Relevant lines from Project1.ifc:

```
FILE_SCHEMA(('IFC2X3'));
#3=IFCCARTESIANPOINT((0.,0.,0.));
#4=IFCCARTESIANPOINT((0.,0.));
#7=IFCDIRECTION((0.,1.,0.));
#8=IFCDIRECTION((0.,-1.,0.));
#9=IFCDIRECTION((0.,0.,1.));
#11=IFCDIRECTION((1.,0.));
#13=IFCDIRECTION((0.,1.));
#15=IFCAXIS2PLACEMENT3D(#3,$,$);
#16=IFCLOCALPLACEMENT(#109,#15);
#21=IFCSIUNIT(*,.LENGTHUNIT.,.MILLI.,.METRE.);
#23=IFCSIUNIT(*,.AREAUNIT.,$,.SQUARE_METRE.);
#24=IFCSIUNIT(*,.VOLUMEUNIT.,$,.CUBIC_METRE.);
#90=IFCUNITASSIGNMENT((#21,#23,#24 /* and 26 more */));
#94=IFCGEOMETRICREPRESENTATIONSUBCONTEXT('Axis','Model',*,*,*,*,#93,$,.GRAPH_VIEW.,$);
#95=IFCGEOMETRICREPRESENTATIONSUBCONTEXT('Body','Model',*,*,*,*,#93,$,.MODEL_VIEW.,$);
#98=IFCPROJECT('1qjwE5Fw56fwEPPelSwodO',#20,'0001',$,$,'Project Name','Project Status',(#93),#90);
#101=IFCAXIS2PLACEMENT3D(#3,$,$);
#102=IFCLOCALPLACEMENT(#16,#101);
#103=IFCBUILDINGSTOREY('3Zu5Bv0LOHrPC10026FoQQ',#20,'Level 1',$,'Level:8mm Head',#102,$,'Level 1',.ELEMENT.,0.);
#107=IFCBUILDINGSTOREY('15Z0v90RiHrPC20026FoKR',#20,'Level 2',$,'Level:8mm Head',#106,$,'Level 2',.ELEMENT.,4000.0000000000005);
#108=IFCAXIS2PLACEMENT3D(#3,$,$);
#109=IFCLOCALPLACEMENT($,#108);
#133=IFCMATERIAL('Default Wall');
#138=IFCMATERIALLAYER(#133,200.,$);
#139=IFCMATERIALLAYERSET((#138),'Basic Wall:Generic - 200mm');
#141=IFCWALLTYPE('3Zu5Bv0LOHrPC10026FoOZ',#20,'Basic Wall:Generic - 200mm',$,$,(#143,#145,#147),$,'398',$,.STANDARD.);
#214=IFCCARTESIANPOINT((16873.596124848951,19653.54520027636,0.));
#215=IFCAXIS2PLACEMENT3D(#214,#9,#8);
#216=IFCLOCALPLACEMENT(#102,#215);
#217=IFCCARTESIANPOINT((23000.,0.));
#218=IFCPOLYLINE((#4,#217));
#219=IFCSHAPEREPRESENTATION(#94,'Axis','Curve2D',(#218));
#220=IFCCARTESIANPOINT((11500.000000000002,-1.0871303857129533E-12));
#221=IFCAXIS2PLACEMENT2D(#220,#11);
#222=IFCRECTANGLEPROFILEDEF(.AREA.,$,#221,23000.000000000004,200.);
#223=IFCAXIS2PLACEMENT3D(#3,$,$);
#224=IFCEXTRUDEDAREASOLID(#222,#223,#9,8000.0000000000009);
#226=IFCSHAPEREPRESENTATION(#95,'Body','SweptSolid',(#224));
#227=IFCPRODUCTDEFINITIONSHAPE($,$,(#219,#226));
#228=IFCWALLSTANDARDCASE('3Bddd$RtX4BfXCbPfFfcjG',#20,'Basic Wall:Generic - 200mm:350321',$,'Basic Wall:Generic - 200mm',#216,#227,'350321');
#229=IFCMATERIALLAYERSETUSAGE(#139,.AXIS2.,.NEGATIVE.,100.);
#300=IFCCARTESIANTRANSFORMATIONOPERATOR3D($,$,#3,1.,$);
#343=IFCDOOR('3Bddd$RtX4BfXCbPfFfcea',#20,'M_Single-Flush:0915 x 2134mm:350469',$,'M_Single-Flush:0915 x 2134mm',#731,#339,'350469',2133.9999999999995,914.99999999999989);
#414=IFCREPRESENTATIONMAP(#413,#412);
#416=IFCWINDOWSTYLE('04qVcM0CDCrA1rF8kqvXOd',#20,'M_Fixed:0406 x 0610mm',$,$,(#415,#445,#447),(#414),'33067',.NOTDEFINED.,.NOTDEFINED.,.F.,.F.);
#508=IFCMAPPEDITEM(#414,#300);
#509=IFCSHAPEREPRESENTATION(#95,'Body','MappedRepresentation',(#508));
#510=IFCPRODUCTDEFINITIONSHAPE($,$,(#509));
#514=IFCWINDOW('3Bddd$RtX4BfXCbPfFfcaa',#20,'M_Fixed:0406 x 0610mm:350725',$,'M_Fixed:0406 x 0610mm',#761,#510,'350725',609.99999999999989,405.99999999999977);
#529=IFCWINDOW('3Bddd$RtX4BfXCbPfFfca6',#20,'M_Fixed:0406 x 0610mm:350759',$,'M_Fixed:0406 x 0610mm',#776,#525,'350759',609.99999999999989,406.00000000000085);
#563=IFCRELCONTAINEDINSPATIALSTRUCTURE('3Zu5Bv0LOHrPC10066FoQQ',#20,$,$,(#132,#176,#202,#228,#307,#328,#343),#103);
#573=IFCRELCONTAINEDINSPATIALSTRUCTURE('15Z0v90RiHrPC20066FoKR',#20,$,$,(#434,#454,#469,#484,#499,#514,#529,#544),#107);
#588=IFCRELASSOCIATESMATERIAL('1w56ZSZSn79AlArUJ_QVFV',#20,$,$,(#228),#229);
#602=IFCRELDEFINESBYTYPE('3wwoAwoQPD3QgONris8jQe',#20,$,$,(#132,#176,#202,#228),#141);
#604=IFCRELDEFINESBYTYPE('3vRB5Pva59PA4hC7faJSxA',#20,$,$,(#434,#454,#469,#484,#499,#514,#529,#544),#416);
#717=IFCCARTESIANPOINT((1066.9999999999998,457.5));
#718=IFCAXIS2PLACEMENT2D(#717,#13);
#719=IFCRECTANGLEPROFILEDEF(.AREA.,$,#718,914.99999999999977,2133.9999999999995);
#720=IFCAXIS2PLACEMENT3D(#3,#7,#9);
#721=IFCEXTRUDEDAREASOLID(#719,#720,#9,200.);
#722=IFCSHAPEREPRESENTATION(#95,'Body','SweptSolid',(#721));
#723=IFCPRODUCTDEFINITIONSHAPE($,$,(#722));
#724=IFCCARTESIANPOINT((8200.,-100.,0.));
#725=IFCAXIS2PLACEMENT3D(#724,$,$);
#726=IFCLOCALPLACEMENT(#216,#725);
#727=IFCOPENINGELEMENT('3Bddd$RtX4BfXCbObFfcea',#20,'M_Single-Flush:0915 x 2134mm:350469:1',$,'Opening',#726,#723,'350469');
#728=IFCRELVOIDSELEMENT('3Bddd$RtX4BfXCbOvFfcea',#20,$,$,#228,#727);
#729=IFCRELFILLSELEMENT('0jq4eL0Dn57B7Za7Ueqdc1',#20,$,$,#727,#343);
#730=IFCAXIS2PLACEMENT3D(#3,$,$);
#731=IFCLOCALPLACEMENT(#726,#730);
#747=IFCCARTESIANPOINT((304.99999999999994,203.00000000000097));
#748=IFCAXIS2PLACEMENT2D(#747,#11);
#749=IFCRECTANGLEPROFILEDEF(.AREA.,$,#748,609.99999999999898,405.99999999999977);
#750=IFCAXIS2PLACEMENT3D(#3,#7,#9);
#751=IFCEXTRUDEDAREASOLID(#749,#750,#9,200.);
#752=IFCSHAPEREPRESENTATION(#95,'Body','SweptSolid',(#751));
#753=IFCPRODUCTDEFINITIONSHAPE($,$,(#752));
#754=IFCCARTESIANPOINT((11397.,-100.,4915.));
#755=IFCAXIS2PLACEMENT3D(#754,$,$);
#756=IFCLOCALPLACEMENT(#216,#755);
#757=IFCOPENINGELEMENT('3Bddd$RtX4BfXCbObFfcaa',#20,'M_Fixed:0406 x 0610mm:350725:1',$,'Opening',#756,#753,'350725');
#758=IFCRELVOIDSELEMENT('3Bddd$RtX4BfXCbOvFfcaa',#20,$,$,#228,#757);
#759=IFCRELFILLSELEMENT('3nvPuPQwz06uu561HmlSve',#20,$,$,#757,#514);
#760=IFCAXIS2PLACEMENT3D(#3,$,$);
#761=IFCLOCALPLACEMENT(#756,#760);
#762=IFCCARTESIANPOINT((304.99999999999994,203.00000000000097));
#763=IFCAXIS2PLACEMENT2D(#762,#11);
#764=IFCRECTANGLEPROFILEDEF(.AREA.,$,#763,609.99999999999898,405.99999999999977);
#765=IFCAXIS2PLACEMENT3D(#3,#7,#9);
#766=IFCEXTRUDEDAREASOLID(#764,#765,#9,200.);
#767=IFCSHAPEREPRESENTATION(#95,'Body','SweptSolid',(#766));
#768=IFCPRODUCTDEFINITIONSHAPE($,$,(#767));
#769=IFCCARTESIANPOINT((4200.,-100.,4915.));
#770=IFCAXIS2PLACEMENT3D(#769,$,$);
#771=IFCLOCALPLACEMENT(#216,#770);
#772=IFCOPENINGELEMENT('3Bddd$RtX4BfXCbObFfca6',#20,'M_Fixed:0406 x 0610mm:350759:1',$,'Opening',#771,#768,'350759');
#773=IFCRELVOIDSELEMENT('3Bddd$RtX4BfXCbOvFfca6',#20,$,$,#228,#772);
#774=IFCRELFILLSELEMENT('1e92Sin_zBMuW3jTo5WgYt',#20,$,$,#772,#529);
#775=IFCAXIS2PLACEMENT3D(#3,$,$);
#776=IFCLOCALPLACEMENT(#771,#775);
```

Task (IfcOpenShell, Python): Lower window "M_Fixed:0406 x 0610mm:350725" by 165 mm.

```python
import numpy as np
import ifcopenshell
import ifcopenshell.api.geometry
import ifcopenshell.util.placement
import ifcopenshell.util.unit

model = ifcopenshell.open("Project1.ifc")
unit_scale = ifcopenshell.util.unit.calculate_unit_scale(model)

window = model.by_id(514)
opening = window.FillsVoids[0].RelatingOpeningElement
dz = -0.165 / unit_scale

shift = np.array([0.0, 0.0, dz])
# The window is placed relative to its opening, so it follows when the opening moves.
matrix = ifcopenshell.util.placement.get_local_placement(opening.ObjectPlacement)
matrix[:3, 3] += shift
ifcopenshell.api.geometry.edit_object_placement(
    model, product=opening, matrix=matrix, is_si=False, should_transform_children=True
)

print(f"moved by {dz * unit_scale:+.3f} m")

model.write("Project1_edited.ifc")
```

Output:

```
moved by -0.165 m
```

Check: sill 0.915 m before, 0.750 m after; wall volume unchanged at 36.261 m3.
